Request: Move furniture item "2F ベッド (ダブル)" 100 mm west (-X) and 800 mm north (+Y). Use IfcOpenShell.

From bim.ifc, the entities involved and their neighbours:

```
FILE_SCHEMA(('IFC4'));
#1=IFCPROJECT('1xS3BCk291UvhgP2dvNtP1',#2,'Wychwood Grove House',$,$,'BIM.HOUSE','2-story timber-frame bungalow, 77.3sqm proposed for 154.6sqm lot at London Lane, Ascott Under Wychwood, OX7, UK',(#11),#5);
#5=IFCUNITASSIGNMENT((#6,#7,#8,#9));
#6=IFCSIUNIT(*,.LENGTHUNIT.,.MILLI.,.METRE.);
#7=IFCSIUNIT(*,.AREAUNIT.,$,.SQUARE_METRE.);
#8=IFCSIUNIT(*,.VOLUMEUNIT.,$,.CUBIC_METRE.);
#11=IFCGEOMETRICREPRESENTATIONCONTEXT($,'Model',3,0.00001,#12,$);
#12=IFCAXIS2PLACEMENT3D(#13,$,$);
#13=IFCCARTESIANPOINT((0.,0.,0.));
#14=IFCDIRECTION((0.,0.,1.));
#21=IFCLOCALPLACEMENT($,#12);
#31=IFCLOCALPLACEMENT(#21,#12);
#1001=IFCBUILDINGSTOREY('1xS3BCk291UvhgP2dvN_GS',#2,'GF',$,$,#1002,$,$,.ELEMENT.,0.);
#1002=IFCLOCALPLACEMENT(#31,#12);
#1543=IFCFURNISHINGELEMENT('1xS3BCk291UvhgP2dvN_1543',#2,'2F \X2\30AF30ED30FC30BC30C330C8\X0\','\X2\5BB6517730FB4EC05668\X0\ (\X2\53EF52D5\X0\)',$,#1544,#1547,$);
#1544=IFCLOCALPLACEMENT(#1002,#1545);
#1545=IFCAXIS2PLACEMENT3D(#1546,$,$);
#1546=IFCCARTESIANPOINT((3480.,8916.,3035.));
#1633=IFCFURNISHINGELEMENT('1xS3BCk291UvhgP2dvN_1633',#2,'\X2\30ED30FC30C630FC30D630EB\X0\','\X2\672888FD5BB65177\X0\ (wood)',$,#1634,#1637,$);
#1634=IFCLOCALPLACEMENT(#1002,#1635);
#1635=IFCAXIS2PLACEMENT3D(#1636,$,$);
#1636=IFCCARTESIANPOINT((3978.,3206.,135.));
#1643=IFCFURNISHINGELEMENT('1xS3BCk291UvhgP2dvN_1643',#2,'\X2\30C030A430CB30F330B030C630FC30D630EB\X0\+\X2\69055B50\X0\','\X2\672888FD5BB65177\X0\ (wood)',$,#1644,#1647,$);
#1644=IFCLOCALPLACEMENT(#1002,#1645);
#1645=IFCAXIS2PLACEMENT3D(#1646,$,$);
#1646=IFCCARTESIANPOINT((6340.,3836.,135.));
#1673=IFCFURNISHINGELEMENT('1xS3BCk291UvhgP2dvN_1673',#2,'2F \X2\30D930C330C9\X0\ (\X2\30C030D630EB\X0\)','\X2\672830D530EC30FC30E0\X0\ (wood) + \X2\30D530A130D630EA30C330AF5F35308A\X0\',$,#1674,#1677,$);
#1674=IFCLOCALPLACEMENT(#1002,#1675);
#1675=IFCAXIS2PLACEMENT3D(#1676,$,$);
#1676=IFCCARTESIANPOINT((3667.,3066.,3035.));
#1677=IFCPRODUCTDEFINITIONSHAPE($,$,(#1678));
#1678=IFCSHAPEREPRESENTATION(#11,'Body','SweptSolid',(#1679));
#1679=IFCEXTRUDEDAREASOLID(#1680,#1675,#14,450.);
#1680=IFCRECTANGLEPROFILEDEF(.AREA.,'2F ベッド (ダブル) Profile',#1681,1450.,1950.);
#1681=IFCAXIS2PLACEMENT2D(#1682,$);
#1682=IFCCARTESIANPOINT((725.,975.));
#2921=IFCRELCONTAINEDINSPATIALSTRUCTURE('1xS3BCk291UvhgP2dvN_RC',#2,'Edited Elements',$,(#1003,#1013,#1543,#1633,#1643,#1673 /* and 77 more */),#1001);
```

```python
import ifcopenshell
import ifcopenshell.api.geometry
import ifcopenshell.util.placement

model = ifcopenshell.open("bim.ifc")

item = model.by_guid("1xS3BCk291UvhgP2dvN_1673")
matrix = ifcopenshell.util.placement.get_local_placement(item.ObjectPlacement)
matrix[0, 3] -= 100.0
matrix[1, 3] += 800.0
ifcopenshell.api.geometry.edit_object_placement(model, product=item, matrix=matrix, is_si=False)

print(ifcopenshell.util.placement.get_local_placement(item.ObjectPlacement).round(3) + 0.0)

model.write("bim_edited.ifc")
```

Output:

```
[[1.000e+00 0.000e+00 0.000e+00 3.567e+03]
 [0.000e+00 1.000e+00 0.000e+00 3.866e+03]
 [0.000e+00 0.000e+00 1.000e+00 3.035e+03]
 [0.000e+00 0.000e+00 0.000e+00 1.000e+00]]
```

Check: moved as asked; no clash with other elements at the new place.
